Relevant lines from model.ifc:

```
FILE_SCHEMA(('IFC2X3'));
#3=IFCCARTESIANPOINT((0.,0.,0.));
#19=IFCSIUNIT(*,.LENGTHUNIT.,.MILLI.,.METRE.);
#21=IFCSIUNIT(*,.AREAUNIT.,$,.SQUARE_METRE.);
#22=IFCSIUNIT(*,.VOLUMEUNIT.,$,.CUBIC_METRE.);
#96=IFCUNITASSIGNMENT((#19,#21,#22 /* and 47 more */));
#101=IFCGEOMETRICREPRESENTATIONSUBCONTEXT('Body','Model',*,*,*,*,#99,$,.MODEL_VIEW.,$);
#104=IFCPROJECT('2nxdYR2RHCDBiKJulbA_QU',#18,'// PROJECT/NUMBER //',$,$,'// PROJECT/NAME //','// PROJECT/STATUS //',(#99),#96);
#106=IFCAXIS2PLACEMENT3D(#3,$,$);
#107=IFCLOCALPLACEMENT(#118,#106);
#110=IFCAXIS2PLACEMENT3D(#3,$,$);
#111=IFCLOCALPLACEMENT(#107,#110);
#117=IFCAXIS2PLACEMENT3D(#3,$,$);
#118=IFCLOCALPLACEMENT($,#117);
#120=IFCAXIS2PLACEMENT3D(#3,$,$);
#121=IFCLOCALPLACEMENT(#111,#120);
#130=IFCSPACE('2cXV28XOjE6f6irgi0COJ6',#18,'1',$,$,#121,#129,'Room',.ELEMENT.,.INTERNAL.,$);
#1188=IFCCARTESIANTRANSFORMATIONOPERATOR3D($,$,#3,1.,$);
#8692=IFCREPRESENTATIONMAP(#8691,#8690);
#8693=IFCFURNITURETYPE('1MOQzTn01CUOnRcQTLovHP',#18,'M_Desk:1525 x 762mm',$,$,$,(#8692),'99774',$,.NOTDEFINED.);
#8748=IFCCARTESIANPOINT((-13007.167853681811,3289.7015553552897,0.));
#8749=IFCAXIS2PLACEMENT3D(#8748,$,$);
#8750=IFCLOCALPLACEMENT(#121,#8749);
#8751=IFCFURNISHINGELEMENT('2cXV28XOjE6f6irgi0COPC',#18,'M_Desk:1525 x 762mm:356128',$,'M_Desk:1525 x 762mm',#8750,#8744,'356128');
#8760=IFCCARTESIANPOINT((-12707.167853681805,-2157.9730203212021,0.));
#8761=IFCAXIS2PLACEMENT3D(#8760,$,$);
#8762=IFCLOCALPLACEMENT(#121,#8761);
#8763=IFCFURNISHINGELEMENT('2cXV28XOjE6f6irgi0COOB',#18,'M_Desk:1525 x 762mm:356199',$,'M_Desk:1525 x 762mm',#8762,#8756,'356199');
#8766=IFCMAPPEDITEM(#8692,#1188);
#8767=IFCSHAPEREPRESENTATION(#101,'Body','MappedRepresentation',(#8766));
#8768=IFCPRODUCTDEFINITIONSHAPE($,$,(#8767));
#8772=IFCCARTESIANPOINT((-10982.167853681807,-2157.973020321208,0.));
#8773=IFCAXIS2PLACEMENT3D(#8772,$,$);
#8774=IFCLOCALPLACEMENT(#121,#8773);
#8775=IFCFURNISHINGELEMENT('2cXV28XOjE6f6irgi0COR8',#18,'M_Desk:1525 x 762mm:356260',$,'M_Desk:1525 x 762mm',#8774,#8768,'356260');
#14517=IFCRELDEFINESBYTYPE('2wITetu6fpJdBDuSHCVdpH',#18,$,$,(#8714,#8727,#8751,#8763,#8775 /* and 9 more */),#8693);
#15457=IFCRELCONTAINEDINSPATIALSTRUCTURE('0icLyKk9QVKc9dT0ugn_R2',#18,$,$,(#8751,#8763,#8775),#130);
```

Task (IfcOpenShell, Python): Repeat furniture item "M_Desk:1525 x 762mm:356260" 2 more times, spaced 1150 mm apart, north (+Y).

```python
import numpy as np
import ifcopenshell
import ifcopenshell.api.geometry
import ifcopenshell.api.root
import ifcopenshell.util.element
import ifcopenshell.util.placement

model = ifcopenshell.open("model.ifc")


def reuse_history(source, copy):
    """copy_class also copies each property set's owner history, people and application; keep the originals."""
    for rel in copy.IsDefinedBy:
        if rel.is_a("IfcRelDefinesByProperties") and (history := rel.RelatingPropertyDefinition.OwnerHistory):
            rel.RelatingPropertyDefinition.OwnerHistory = source.OwnerHistory
            ifcopenshell.util.element.remove_deep2(model, history)


source = model.by_guid("2cXV28XOjE6f6irgi0COR8")
base = ifcopenshell.util.placement.get_local_placement(source.ObjectPlacement)
step = np.array([0.0, 1.0, 0.0]) * 1150.0

for i in range(1, 3):
    copy = ifcopenshell.api.root.copy_class(model, product=source)
    copy.Representation = ifcopenshell.util.element.copy_deep(
        model, source.Representation, exclude=["IfcGeometricRepresentationContext", "IfcRepresentationMap"]
    )
    copy.Name = "M_Desk:1525 x 762mm"
    copy.Tag = None
    reuse_history(source, copy)
    matrix = base.copy()
    matrix[:3, 3] += i * step
    print("added at", matrix[:3, 3].round(3) + 0.0)
    ifcopenshell.api.geometry.edit_object_placement(model, product=copy, matrix=matrix, is_si=False)

model.write("model_updated.ifc")
```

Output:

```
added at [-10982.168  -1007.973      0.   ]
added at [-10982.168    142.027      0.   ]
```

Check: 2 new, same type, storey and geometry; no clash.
